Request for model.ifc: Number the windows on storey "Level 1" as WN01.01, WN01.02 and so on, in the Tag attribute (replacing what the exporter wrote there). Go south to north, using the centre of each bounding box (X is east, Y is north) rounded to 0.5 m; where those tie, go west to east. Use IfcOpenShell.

First a look at what the model holds.

```python
import ifcopenshell
import ifcopenshell.util.element
import ifcopenshell.util.placement

model = ifcopenshell.open("model.ifc")
print(model.schema)
storey = next(s for s in model.by_type("IfcBuildingStorey") if s.Name == "Level 1")
windows = [e for e in ifcopenshell.util.element.get_decomposition(storey) if e.is_a("IfcWindow")]
for e in sorted(windows, key=lambda e: e.id()):
    origin = ifcopenshell.util.placement.get_local_placement(e.ObjectPlacement)[:3, 3]
    print(e.id(), e.Tag, e.Name, origin.round(2) + 0.0, sep=" | ")
```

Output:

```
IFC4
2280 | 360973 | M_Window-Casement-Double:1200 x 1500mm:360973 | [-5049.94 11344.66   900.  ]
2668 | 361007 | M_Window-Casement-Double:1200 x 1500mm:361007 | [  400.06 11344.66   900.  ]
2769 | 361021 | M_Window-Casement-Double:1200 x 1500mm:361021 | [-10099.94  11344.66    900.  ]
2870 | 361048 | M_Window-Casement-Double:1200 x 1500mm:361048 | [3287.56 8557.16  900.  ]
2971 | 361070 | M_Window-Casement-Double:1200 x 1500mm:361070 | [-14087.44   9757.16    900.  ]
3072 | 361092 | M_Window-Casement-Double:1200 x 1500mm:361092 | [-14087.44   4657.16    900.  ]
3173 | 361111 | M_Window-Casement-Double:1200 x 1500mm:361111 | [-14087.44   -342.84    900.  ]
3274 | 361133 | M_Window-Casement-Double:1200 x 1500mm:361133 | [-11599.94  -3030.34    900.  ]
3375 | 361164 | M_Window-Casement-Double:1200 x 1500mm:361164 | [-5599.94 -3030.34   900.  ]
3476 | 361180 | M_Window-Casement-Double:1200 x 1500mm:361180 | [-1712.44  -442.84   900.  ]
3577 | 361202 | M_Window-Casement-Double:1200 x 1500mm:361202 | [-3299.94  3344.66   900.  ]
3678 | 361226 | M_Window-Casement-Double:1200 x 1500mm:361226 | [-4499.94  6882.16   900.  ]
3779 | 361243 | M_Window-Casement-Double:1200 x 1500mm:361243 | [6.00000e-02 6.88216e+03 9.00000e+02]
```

```python
import ifcopenshell
import ifcopenshell.geom
import ifcopenshell.util.element
import ifcopenshell.util.shape

model = ifcopenshell.open("model.ifc")
settings = ifcopenshell.geom.settings()
settings.set("use-world-coords", True)


def centre(element):
    shape = ifcopenshell.geom.create_shape(settings, element)
    return ifcopenshell.util.shape.get_bbox_centroid(shape.geometry)


storey = next(s for s in model.by_type("IfcBuildingStorey") if s.Name == "Level 1")
windows = [e for e in ifcopenshell.util.element.get_decomposition(storey) if e.is_a("IfcWindow")]

# Insertion points can sit at a corner or the storey origin, so sort by the geometry (in metres).
centres = {e: centre(e) for e in windows}
windows.sort(key=lambda e: (round(centres[e][1] / 0.5), centres[e][0]))

for i, e in enumerate(windows, start=1):
    number = f"WN01.{i:02d}"
    e.Tag = number
    print(e.id(), number)

model.write("model_edited.ifc")
```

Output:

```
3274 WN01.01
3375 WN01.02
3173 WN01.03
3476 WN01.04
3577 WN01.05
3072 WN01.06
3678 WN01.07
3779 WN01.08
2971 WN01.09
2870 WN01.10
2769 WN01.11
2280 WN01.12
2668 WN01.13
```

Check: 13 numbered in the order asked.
